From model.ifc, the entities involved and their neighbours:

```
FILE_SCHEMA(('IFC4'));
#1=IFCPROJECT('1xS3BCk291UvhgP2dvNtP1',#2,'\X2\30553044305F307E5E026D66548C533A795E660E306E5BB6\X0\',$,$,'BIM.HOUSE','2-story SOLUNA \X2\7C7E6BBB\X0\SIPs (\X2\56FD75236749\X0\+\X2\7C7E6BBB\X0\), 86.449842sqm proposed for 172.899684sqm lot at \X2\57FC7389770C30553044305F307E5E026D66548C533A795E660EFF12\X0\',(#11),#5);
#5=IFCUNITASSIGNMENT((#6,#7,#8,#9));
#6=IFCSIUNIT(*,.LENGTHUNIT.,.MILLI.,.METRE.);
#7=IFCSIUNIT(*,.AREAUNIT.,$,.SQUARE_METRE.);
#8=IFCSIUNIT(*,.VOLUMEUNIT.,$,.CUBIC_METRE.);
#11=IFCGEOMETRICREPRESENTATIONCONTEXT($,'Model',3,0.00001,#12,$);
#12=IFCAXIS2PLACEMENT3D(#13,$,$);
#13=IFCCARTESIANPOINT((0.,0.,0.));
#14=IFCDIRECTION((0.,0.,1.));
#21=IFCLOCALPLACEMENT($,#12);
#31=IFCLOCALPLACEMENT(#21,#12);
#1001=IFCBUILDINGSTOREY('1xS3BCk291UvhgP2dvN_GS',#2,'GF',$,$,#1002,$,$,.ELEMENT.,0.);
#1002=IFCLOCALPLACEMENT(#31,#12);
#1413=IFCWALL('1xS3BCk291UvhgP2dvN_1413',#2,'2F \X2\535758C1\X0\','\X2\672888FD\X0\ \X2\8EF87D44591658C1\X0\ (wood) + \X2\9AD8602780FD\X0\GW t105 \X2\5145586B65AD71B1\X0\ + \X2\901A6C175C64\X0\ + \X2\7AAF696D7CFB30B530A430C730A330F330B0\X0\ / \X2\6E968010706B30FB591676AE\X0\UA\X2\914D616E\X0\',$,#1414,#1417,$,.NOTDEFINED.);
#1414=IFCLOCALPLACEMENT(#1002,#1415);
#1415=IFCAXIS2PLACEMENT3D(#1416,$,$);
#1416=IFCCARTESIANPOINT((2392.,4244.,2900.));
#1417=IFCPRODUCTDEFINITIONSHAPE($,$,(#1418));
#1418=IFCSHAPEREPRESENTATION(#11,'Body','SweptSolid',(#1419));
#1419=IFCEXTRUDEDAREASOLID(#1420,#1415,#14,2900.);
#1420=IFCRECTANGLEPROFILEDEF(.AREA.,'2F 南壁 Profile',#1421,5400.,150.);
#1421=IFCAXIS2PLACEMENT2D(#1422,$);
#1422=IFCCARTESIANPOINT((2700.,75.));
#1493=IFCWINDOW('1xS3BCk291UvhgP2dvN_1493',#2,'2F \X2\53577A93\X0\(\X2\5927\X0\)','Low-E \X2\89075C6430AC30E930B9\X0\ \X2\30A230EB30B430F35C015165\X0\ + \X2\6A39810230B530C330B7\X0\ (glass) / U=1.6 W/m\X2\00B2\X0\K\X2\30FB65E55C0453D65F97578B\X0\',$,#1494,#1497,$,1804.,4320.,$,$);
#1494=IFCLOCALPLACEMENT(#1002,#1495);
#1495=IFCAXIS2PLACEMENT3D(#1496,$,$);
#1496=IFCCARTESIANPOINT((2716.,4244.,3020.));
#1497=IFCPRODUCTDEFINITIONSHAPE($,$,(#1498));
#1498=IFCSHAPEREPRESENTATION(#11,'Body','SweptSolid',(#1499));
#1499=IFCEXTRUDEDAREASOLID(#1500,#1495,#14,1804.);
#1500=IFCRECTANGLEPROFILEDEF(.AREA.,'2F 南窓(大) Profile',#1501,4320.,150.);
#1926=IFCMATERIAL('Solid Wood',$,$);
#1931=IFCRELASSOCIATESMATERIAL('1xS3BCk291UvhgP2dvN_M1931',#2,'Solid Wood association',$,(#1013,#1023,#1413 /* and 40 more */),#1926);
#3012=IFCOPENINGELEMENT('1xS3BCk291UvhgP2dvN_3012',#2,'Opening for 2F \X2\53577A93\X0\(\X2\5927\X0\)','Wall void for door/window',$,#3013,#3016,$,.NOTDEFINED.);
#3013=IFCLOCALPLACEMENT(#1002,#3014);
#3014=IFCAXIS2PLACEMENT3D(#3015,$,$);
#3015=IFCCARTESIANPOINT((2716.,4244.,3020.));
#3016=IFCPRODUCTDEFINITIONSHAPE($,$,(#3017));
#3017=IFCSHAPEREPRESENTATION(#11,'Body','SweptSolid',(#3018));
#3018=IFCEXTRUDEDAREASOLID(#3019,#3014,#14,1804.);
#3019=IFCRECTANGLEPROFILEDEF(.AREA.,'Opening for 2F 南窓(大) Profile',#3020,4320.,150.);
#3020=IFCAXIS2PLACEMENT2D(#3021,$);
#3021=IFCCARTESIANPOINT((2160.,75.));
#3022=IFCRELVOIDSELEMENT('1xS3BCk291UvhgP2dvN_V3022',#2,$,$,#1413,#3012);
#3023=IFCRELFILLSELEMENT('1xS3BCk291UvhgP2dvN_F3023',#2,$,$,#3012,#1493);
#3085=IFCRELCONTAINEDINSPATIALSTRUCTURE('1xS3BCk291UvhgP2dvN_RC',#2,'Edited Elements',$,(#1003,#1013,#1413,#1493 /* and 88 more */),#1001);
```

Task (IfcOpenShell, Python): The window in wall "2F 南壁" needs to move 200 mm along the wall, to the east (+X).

```python
import ifcopenshell
import ifcopenshell.api.geometry
import ifcopenshell.util.placement
import ifcopenshell.util.unit

model = ifcopenshell.open("model.ifc")
unit_scale = ifcopenshell.util.unit.calculate_unit_scale(model)

window = model.by_guid("1xS3BCk291UvhgP2dvN_1493")
opening = window.FillsVoids[0].RelatingOpeningElement
wall = opening.VoidsElements[0].RelatingBuildingElement

wall_matrix = ifcopenshell.util.placement.get_local_placement(wall.ObjectPlacement)
shift = wall_matrix[:3, 0] * 0.2 / unit_scale
before = ifcopenshell.util.placement.get_local_placement(window.ObjectPlacement)[:3, 3].copy()

# The window is not placed relative to its opening, so move both.
for product in (opening, window):
    matrix = ifcopenshell.util.placement.get_local_placement(product.ObjectPlacement)
    matrix[:3, 3] += shift
    ifcopenshell.api.geometry.edit_object_placement(model, product=product, matrix=matrix, is_si=False)

after = ifcopenshell.util.placement.get_local_placement(window.ObjectPlacement)[:3, 3]
print("window moved by", (after - before).round(3) + 0.0)

model.write("model_updated.ifc")
```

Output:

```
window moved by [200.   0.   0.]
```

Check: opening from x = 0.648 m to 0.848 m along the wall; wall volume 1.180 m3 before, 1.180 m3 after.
